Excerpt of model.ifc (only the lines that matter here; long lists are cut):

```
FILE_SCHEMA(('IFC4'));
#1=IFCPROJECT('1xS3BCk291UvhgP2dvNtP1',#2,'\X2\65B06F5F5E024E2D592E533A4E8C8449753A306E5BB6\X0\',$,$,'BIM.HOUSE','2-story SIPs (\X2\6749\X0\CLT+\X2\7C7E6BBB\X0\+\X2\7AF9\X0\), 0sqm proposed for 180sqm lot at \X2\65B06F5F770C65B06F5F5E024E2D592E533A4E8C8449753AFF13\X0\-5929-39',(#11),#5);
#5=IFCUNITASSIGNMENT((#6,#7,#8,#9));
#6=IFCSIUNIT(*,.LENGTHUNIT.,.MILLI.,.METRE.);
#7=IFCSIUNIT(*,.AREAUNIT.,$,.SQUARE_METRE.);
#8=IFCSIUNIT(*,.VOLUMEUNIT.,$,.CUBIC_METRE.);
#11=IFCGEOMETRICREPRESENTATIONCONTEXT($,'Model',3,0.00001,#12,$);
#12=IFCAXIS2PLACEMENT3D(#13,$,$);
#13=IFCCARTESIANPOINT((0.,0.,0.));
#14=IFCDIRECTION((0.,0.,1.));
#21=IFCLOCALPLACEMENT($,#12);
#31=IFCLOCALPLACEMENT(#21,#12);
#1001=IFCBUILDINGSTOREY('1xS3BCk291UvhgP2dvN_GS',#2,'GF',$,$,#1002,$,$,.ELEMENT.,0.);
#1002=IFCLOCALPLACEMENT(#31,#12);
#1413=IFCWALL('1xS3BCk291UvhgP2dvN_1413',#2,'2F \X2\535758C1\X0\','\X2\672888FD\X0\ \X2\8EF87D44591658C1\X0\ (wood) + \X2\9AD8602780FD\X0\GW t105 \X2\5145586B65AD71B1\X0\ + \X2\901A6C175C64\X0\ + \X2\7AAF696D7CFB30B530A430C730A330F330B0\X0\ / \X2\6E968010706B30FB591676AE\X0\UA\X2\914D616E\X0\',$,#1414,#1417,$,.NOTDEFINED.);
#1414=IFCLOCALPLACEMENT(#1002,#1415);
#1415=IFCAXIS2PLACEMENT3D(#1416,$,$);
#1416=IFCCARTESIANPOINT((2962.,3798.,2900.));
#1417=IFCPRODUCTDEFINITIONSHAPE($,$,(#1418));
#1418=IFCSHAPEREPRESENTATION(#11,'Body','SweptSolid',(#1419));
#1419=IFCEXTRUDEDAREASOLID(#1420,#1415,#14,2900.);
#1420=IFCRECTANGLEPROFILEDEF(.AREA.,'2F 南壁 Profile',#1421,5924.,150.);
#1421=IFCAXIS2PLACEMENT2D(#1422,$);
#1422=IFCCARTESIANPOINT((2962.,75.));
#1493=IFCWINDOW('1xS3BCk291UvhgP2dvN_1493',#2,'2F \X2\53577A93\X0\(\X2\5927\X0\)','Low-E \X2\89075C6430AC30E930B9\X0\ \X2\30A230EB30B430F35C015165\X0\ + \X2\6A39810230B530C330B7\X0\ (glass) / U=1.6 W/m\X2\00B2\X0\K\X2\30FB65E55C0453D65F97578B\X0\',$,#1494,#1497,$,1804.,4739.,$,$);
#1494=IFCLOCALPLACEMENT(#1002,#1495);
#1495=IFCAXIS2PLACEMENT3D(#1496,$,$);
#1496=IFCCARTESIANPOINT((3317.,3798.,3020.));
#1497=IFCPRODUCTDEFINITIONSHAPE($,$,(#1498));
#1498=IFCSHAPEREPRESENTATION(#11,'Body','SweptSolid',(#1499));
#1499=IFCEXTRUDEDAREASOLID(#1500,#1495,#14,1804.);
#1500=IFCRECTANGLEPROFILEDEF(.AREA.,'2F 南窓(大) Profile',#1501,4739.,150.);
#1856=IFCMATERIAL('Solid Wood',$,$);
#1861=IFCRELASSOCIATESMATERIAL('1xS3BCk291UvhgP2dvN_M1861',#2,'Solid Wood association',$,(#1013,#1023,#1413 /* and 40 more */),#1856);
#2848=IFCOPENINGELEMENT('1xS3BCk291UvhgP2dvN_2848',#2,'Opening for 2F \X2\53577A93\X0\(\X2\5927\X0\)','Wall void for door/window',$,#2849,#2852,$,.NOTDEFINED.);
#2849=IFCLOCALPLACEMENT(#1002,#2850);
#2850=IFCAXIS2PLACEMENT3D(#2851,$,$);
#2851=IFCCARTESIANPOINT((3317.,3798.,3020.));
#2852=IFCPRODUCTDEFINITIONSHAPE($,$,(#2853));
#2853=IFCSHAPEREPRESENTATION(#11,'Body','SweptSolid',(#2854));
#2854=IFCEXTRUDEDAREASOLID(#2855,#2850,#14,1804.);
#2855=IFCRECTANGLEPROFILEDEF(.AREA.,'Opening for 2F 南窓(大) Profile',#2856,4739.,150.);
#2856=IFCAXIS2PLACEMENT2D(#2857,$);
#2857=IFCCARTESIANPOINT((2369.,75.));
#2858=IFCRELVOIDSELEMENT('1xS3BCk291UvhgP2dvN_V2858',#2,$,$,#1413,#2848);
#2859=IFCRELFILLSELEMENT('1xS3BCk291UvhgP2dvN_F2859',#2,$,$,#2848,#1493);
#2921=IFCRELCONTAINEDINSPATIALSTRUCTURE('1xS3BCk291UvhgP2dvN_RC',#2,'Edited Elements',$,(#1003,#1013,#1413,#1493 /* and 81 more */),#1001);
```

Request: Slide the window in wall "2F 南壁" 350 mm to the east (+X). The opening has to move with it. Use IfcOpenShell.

```python
import ifcopenshell
import ifcopenshell.api.geometry
import ifcopenshell.util.placement
import ifcopenshell.util.unit

model = ifcopenshell.open("model.ifc")
unit_scale = ifcopenshell.util.unit.calculate_unit_scale(model)

window = model.by_id(1493)
opening = window.FillsVoids[0].RelatingOpeningElement
wall = opening.VoidsElements[0].RelatingBuildingElement

wall_matrix = ifcopenshell.util.placement.get_local_placement(wall.ObjectPlacement)
shift = wall_matrix[:3, 0] * 0.35 / unit_scale
before = ifcopenshell.util.placement.get_local_placement(window.ObjectPlacement)[:3, 3].copy()

# The window is not placed relative to its opening, so move both.
for product in (opening, window):
    matrix = ifcopenshell.util.placement.get_local_placement(product.ObjectPlacement)
    matrix[:3, 3] += shift
    ifcopenshell.api.geometry.edit_object_placement(model, product=product, matrix=matrix, is_si=False)

after = ifcopenshell.util.placement.get_local_placement(window.ObjectPlacement)[:3, 3]
print("window moved by", (after - before).round(3) + 0.0)

model.write("model_updated.ifc")
```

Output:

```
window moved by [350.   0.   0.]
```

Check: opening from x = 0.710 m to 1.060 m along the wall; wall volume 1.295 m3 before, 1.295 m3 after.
